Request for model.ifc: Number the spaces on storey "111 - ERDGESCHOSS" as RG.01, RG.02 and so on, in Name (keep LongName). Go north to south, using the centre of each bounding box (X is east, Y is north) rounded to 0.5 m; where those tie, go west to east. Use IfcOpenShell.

First a look at what the model holds.

```python
import ifcopenshell
import ifcopenshell.util.element
import ifcopenshell.util.placement

model = ifcopenshell.open("model.ifc")
print(model.schema)
storey = next(s for s in model.by_type("IfcBuildingStorey") if s.Name == "111 - ERDGESCHOSS")
spaces = [e for e in ifcopenshell.util.element.get_decomposition(storey) if e.is_a("IfcSpace")]
for e in sorted(spaces, key=lambda e: e.id()):
    origin = ifcopenshell.util.placement.get_local_placement(e.ObjectPlacement)[:3, 3]
    print(e.id(), e.Name, e.LongName, origin.round(2) + 0.0, sep=" | ")
```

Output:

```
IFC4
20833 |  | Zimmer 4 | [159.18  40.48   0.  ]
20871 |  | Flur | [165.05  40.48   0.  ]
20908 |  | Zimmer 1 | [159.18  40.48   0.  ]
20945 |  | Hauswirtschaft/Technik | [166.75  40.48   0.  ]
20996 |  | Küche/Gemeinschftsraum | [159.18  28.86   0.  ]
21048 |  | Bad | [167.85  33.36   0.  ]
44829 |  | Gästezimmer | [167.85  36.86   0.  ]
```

```python
import ifcopenshell
import ifcopenshell.geom
import ifcopenshell.util.element
import ifcopenshell.util.shape

model = ifcopenshell.open("model.ifc")
settings = ifcopenshell.geom.settings()
settings.set("use-world-coords", True)


def centre(element):
    shape = ifcopenshell.geom.create_shape(settings, element)
    return ifcopenshell.util.shape.get_bbox_centroid(shape.geometry)


storey = next(s for s in model.by_type("IfcBuildingStorey") if s.Name == "111 - ERDGESCHOSS")
spaces = [e for e in ifcopenshell.util.element.get_decomposition(storey) if e.is_a("IfcSpace")]

# Insertion points can sit at a corner or the storey origin, so sort by the geometry (in metres).
centres = {e: centre(e) for e in spaces}
spaces.sort(key=lambda e: (-round(centres[e][1] / 0.5), centres[e][0]))

for i, e in enumerate(spaces, start=1):
    number = f"RG.{i:02d}"
    e.Name = number
    print(e.id(), number)

model.write("model_updated.ifc")
```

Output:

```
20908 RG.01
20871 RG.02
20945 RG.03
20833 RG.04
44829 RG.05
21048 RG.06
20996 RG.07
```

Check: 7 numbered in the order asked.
